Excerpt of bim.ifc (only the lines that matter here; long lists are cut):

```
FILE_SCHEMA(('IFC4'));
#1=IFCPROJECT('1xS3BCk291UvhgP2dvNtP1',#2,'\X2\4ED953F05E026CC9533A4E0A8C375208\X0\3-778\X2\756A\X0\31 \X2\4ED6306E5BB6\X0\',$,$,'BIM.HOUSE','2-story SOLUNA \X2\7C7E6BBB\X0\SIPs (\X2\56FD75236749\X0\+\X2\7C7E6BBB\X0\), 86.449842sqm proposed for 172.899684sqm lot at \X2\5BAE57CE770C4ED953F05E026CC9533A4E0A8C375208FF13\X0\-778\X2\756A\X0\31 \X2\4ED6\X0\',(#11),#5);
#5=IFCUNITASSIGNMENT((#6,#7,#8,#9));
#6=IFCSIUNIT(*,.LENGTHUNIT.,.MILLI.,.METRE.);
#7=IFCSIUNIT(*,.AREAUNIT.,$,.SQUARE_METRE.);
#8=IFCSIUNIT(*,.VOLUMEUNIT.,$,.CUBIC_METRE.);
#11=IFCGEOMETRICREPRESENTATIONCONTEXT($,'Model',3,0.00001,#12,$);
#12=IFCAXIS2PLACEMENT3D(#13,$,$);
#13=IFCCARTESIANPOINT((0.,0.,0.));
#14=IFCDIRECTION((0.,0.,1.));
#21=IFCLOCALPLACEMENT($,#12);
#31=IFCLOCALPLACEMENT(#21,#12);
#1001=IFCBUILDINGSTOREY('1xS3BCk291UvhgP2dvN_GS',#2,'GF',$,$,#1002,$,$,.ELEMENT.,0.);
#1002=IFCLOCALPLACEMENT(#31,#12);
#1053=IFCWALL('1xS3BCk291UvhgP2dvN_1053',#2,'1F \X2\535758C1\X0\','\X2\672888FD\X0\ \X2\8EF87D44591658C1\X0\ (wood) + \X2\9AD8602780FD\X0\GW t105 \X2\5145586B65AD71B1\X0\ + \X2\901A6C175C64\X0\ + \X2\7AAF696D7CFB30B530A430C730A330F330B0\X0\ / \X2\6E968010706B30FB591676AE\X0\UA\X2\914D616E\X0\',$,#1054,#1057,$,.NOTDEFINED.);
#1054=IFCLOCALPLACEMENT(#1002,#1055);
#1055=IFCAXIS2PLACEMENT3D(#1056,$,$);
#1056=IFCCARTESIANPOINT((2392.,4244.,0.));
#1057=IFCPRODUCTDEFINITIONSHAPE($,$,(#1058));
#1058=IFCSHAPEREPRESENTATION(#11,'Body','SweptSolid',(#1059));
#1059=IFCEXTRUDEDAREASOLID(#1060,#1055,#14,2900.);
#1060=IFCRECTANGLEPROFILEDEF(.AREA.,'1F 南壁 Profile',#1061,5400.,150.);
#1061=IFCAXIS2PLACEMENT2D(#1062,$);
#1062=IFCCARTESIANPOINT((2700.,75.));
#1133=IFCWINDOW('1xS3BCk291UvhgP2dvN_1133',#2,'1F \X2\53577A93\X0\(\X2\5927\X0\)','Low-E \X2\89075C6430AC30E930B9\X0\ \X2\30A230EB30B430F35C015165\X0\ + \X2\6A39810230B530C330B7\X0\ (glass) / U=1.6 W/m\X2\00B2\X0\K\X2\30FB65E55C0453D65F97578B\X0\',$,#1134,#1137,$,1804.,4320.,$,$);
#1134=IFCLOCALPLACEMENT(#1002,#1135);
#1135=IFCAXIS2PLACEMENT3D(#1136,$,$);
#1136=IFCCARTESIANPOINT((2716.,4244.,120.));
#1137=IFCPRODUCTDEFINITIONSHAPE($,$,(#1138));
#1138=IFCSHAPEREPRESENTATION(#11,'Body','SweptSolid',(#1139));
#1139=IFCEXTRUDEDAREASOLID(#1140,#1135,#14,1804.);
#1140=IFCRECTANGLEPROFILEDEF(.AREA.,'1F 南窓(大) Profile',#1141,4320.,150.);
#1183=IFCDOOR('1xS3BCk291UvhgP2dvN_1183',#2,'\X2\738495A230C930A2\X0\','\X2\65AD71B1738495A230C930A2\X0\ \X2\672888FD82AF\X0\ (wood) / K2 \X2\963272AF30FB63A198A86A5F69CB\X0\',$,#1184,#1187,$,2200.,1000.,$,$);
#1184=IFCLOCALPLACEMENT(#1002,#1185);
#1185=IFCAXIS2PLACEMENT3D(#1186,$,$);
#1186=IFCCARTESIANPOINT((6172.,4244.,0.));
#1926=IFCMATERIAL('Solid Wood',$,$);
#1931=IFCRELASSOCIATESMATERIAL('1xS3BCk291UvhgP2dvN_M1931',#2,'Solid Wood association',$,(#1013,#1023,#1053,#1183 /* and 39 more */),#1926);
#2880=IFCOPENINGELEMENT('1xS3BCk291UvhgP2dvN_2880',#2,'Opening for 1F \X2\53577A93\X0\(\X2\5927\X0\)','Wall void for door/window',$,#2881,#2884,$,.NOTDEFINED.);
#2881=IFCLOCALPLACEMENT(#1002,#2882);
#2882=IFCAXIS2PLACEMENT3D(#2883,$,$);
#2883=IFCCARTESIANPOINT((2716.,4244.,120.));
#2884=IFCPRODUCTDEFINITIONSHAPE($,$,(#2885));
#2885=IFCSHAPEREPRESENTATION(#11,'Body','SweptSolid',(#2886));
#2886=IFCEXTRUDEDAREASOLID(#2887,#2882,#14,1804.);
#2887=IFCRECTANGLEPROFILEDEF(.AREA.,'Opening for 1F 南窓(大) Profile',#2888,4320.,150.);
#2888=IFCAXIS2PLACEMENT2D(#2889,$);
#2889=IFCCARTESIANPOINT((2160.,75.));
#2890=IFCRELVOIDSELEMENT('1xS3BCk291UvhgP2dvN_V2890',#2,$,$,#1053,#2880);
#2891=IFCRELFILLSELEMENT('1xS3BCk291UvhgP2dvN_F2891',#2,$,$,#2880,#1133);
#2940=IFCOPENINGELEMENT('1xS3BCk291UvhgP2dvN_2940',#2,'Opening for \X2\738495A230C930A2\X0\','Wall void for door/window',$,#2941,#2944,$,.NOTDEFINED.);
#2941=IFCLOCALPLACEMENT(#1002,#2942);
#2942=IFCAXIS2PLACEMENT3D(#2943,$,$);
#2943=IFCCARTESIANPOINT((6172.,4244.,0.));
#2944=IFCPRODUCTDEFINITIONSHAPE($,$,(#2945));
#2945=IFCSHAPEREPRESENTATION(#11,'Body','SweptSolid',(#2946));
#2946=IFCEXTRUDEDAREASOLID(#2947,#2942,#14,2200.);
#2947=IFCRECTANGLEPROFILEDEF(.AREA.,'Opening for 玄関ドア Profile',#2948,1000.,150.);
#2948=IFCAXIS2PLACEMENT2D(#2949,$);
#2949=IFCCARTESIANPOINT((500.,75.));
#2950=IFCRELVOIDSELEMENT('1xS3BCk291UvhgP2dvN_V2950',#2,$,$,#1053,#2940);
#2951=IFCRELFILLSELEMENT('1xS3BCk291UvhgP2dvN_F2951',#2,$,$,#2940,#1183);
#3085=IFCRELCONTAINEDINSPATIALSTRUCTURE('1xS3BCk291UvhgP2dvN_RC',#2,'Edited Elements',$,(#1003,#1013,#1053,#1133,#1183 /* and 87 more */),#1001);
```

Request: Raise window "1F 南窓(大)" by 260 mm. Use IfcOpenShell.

```python
import numpy as np
import ifcopenshell
import ifcopenshell.api.geometry
import ifcopenshell.util.placement
import ifcopenshell.util.unit

model = ifcopenshell.open("bim.ifc")
unit_scale = ifcopenshell.util.unit.calculate_unit_scale(model)

window = model.by_guid("1xS3BCk291UvhgP2dvN_1133")
opening = window.FillsVoids[0].RelatingOpeningElement
dz = 260.0

shift = np.array([0.0, 0.0, dz])
# The window is not placed relative to its opening, so move both.
for product in (opening, window):
    matrix = ifcopenshell.util.placement.get_local_placement(product.ObjectPlacement)
    matrix[:3, 3] += shift
    ifcopenshell.api.geometry.edit_object_placement(model, product=product, matrix=matrix, is_si=False)

print(f"moved by {dz * unit_scale:+.3f} m")

model.write("bim-out.ifc")
```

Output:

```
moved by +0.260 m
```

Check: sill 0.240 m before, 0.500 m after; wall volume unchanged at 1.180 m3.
